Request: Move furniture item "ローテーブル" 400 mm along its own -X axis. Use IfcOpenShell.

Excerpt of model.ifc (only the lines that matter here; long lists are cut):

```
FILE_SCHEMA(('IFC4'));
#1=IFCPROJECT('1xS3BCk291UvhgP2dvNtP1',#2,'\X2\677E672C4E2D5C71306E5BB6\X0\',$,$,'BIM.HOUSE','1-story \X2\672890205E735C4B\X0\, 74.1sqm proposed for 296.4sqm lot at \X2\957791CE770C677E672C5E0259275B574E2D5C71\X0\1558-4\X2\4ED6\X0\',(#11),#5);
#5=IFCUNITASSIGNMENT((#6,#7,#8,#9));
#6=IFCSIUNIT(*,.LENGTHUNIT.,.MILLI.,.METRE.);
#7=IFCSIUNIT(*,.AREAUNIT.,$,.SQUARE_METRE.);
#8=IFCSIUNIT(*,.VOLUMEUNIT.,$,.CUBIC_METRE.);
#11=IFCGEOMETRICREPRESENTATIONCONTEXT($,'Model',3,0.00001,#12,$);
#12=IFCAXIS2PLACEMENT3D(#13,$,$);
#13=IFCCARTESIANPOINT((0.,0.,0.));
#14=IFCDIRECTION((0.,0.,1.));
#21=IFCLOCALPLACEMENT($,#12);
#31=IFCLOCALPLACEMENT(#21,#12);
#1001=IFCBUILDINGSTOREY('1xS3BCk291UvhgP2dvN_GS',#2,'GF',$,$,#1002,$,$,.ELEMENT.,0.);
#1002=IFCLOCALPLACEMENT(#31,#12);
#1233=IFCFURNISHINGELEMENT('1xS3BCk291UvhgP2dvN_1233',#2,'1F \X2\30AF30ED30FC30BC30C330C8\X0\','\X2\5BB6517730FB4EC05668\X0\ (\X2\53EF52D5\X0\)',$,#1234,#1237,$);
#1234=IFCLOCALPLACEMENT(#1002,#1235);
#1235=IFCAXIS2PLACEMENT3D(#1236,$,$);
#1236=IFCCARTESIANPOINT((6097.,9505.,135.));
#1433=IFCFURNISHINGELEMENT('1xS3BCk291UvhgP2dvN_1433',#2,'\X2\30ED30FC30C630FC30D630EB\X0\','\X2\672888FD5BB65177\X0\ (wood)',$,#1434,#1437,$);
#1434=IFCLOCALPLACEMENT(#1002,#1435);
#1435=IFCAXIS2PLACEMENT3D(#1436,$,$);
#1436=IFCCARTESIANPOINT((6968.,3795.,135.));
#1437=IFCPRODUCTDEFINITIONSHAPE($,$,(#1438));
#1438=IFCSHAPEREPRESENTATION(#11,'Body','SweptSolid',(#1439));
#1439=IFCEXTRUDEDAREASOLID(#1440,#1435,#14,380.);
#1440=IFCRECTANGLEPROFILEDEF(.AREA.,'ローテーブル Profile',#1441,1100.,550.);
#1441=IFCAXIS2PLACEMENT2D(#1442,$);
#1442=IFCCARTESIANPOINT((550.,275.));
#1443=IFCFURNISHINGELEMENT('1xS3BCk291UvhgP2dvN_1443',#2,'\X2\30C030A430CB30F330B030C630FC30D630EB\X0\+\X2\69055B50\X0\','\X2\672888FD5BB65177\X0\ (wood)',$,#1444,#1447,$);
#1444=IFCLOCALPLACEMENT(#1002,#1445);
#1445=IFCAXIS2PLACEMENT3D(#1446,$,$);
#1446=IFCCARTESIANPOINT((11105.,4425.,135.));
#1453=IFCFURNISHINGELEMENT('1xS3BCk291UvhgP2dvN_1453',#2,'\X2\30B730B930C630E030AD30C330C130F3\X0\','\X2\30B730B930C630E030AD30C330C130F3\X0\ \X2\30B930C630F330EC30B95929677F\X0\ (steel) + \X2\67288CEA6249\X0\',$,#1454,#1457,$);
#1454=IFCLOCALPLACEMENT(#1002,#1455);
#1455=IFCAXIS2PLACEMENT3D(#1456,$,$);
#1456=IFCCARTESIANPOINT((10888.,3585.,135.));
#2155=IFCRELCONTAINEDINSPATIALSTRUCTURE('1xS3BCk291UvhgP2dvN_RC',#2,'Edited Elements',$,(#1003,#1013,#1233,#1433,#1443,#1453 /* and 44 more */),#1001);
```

```python
import ifcopenshell
import ifcopenshell.api.geometry
import ifcopenshell.util.placement
import ifcopenshell.util.unit

model = ifcopenshell.open("model.ifc")
unit_scale = ifcopenshell.util.unit.calculate_unit_scale(model)

item = model.by_guid("1xS3BCk291UvhgP2dvN_1433")
matrix = ifcopenshell.util.placement.get_local_placement(item.ObjectPlacement)
matrix[:3, 3] -= matrix[:3, 0] * 0.4 / unit_scale
ifcopenshell.api.geometry.edit_object_placement(model, product=item, matrix=matrix, is_si=False)

print(ifcopenshell.util.placement.get_local_placement(item.ObjectPlacement).round(3) + 0.0)

model.write("model-out.ifc")
```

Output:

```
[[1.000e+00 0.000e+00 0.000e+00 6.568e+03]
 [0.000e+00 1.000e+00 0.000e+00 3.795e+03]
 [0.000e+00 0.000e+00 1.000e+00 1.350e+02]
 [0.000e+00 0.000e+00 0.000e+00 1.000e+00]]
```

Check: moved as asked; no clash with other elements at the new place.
